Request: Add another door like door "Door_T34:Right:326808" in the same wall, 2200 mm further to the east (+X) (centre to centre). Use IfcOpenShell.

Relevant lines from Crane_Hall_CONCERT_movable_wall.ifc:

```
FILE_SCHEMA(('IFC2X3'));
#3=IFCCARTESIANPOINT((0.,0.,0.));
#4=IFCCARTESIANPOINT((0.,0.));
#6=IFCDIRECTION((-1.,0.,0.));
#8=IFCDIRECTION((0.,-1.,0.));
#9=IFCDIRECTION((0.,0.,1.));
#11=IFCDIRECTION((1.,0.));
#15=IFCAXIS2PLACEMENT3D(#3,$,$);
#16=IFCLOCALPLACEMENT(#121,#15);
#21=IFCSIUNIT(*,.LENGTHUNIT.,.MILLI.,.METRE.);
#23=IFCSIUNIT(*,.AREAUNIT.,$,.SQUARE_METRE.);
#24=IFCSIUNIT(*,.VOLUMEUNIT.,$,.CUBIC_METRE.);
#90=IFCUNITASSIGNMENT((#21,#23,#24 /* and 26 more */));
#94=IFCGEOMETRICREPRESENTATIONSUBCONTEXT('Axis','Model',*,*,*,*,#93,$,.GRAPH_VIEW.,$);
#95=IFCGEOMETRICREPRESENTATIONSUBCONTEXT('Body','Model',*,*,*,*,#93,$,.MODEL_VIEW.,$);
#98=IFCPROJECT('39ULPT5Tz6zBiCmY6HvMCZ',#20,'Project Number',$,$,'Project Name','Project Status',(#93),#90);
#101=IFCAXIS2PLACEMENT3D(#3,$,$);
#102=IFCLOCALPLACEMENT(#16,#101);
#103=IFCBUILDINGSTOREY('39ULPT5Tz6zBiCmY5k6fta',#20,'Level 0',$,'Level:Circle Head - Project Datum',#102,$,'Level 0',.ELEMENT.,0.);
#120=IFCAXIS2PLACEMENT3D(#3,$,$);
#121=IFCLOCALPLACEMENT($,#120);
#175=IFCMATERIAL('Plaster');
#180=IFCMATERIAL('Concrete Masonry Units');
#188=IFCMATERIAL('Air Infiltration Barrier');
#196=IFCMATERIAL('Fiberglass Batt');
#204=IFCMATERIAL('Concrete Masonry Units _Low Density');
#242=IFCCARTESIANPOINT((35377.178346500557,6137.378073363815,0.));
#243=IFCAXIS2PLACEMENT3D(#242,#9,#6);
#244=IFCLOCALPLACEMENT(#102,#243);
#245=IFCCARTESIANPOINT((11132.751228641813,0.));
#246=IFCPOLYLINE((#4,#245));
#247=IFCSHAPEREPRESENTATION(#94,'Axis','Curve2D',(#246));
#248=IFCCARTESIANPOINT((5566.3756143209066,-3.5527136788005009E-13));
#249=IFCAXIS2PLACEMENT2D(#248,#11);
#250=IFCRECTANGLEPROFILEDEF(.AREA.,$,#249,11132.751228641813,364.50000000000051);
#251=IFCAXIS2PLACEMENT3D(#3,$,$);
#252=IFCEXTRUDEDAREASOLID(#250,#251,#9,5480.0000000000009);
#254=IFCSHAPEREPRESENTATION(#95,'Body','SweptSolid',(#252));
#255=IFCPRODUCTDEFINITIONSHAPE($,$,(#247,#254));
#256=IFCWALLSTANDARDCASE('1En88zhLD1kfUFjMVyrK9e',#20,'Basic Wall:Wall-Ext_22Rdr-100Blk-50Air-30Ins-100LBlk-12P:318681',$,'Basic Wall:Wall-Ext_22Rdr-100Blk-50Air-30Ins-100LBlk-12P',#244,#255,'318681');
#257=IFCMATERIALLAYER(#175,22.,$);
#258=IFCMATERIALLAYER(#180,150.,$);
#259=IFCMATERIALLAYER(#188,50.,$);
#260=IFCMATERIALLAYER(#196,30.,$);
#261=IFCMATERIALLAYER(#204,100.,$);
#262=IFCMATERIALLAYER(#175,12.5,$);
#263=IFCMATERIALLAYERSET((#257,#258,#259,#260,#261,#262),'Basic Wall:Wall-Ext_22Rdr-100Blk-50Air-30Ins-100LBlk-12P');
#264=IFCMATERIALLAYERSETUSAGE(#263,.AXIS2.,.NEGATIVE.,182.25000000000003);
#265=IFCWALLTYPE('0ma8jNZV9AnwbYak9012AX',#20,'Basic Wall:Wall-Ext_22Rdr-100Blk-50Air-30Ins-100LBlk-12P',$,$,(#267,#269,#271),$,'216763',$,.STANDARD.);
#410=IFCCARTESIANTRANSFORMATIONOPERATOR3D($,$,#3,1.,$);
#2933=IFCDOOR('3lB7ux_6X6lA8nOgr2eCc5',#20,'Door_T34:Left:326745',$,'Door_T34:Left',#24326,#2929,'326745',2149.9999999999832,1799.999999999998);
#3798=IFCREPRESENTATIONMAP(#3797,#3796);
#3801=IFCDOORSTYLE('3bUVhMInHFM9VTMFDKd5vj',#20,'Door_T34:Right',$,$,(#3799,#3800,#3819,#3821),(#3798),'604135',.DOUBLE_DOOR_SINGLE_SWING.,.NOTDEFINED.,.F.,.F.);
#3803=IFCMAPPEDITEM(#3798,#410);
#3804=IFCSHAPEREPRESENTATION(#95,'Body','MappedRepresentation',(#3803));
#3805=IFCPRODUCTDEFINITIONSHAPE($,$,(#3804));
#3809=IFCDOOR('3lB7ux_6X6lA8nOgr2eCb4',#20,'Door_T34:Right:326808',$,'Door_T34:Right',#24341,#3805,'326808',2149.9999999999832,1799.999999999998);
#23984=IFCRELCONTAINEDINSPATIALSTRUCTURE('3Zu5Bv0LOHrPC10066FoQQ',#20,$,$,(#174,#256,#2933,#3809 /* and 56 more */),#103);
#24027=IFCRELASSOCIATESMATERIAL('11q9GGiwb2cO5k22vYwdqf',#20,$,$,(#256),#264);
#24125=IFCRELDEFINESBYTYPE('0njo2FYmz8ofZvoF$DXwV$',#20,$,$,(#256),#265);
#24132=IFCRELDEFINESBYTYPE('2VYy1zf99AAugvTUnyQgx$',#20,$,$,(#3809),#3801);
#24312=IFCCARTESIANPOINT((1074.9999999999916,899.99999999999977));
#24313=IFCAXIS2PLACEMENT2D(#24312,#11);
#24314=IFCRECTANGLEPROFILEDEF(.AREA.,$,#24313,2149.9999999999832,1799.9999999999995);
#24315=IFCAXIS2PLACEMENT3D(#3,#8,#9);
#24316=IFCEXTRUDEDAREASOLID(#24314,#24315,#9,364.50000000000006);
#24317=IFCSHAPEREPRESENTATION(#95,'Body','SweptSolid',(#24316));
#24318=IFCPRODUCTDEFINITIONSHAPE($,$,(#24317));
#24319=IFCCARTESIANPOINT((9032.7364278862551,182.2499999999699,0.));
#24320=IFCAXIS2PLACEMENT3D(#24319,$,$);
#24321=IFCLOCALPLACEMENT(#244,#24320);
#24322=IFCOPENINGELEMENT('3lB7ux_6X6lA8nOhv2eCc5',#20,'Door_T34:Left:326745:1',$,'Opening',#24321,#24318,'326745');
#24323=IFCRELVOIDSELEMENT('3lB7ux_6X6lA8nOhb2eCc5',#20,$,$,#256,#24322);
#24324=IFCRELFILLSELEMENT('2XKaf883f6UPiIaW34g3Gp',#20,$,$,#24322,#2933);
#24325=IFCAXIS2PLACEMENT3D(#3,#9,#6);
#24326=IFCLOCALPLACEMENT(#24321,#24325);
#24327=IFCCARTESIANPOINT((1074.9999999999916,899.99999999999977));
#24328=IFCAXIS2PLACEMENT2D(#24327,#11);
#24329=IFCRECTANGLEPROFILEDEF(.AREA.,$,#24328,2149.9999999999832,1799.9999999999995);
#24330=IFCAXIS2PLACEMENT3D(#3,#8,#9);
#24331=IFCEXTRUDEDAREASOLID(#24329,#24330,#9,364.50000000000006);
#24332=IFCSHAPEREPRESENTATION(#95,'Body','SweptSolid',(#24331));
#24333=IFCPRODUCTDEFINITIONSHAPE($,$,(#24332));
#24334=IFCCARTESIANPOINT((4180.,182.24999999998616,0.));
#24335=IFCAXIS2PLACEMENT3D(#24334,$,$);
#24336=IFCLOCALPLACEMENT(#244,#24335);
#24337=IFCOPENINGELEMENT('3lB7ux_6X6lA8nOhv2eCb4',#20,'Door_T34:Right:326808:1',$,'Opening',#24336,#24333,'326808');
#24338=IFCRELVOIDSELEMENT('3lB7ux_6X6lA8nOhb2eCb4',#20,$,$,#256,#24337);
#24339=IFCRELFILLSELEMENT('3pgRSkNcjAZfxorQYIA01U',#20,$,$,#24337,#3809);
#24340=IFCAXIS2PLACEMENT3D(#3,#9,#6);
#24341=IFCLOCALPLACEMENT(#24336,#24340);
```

```python
import ifcopenshell
import ifcopenshell.api.feature
import ifcopenshell.api.geometry
import ifcopenshell.api.root
import ifcopenshell.geom
import ifcopenshell.util.element
import ifcopenshell.util.placement
import ifcopenshell.util.shape

model = ifcopenshell.open("Crane_Hall_CONCERT_movable_wall.ifc")
settings = ifcopenshell.geom.settings()


def volume(element):
    """Net volume in cubic metres, openings subtracted."""
    shape = ifcopenshell.geom.create_shape(settings, element)
    return ifcopenshell.util.shape.get_volume(shape.geometry)


def reuse_history(source, copy):
    """copy_class also copies each property set's owner history, people and application; keep the originals."""
    for rel in copy.IsDefinedBy:
        if rel.is_a("IfcRelDefinesByProperties") and (history := rel.RelatingPropertyDefinition.OwnerHistory):
            rel.RelatingPropertyDefinition.OwnerHistory = source.OwnerHistory
            ifcopenshell.util.element.remove_deep2(model, history)


door = model.by_id(3809)
opening = door.FillsVoids[0].RelatingOpeningElement
wall = opening.VoidsElements[0].RelatingBuildingElement
before = volume(wall)
shift = ifcopenshell.util.placement.get_local_placement(wall.ObjectPlacement)[:3, 0] * -2200.0

# copy_class copies the void relationship, type, container and properties, but no geometry.
new_opening = ifcopenshell.api.root.copy_class(model, product=opening)
new_opening.Representation = ifcopenshell.util.element.copy_deep(
    model, opening.Representation, exclude=["IfcGeometricRepresentationContext", "IfcRepresentationMap"]
)
new_opening.Name = "Door_T34:Right"
new_opening.Tag = None
new_door = ifcopenshell.api.root.copy_class(model, product=door)
new_door.Representation = ifcopenshell.util.element.copy_deep(
    model, door.Representation, exclude=["IfcGeometricRepresentationContext", "IfcRepresentationMap"]
)
new_door.Name = "Door_T34:Right"
new_door.Tag = None
reuse_history(door, new_door)
fills = ifcopenshell.api.feature.add_filling(model, opening=new_opening, element=new_door)
fills.OwnerHistory = new_door.OwnerHistory  # required in IFC2X3

for old, new in ((opening, new_opening), (door, new_door)):
    matrix = ifcopenshell.util.placement.get_local_placement(old.ObjectPlacement)
    matrix[:3, 3] += shift
    ifcopenshell.api.geometry.edit_object_placement(model, product=new, matrix=matrix, is_si=False)

after = volume(wall)

print(f"wall volume {before:.3f} -> {after:.3f} m3")

model.write("Crane_Hall_CONCERT_movable_wall_rev.ifc")
```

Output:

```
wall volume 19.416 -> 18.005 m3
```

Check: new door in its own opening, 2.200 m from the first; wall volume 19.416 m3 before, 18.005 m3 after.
